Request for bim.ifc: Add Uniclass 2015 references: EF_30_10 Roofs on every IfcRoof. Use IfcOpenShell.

First a look at what the model holds.

```python
import ifcopenshell

model = ifcopenshell.open("bim.ifc")
print(model.schema)
print("classifications:", [c.Name for c in model.by_type("IfcClassification")])
for ifc_class in ("IfcDoor", "IfcRoof", "IfcStair", "IfcWall", "IfcWindow"):
    print(ifc_class, len(model.by_type(ifc_class)))
```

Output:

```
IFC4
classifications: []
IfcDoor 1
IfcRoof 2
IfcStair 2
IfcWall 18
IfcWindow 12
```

```python
import ifcopenshell
import ifcopenshell.api.classification

model = ifcopenshell.open("bim.ifc")

system = ifcopenshell.api.classification.add_classification(model, classification="Uniclass 2015")

codes = {
    "IfcRoof": ("EF_30_10", "Roofs"),
}
for ifc_class, (code, name) in codes.items():
    products = model.by_type(ifc_class)
    ifcopenshell.api.classification.add_reference(
        model, products=products, classification=system, identification=code, name=name
    )
    print(code, len(products))

model.write("bim_updated.ifc")
```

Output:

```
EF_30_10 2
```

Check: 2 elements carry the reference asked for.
